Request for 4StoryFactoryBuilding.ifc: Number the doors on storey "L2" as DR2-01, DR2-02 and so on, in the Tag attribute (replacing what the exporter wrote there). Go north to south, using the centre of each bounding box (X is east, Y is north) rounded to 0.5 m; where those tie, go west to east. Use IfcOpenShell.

First a look at what the model holds.

```python
import ifcopenshell
import ifcopenshell.util.element
import ifcopenshell.util.placement

model = ifcopenshell.open("4StoryFactoryBuilding.ifc")
print(model.schema)
storey = next(s for s in model.by_type("IfcBuildingStorey") if s.Name == "L2")
doors = [e for e in ifcopenshell.util.element.get_decomposition(storey) if e.is_a("IfcDoor")]
for e in sorted(doors, key=lambda e: e.id()):
    origin = ifcopenshell.util.placement.get_local_placement(e.ObjectPlacement)[:3, 3]
    print(e.id(), e.Tag, e.Name, origin.round(2) + 0.0, sep=" | ")
```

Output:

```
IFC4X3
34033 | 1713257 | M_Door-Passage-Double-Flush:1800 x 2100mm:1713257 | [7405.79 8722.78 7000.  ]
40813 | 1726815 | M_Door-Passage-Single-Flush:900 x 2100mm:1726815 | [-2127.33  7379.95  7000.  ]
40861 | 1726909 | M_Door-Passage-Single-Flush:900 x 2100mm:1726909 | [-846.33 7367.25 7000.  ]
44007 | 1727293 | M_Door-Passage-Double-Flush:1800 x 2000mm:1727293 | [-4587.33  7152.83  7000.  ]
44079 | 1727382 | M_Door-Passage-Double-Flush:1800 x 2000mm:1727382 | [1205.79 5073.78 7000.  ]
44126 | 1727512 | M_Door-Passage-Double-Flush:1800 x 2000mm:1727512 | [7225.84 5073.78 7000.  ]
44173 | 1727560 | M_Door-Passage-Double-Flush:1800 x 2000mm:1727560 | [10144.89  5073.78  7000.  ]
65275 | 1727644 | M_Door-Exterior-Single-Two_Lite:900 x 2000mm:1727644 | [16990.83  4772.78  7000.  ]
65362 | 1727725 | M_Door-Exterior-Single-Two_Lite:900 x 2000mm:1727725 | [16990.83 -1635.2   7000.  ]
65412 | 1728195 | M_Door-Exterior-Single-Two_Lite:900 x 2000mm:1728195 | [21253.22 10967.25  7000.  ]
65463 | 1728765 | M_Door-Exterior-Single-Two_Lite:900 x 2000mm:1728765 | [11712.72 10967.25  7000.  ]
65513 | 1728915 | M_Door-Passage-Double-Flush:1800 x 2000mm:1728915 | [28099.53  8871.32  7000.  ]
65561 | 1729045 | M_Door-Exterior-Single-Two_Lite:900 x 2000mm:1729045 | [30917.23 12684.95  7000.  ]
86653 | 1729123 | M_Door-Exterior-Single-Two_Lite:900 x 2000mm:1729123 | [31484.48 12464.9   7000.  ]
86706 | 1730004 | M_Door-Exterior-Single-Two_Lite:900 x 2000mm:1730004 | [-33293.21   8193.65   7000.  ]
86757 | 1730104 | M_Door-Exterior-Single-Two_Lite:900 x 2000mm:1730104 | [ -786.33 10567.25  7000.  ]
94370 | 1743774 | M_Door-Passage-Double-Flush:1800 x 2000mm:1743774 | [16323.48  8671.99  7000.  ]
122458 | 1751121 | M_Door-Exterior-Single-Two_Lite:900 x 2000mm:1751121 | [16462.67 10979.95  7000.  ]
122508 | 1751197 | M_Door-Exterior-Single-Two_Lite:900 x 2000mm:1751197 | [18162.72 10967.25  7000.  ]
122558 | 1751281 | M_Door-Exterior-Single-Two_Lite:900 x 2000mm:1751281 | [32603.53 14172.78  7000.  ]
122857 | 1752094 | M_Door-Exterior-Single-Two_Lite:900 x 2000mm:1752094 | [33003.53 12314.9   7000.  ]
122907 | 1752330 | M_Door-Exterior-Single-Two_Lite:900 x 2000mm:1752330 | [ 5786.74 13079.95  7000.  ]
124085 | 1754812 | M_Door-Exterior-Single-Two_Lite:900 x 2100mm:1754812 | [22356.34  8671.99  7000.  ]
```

```python
import ifcopenshell
import ifcopenshell.geom
import ifcopenshell.util.element
import ifcopenshell.util.shape

model = ifcopenshell.open("4StoryFactoryBuilding.ifc")
settings = ifcopenshell.geom.settings()
settings.set("use-world-coords", True)


def centre(element):
    shape = ifcopenshell.geom.create_shape(settings, element)
    return ifcopenshell.util.shape.get_bbox_centroid(shape.geometry)


storey = next(s for s in model.by_type("IfcBuildingStorey") if s.Name == "L2")
doors = [e for e in ifcopenshell.util.element.get_decomposition(storey) if e.is_a("IfcDoor")]

# Insertion points can sit at a corner or the storey origin, so sort by the geometry (in metres).
centres = {e: centre(e) for e in doors}
doors.sort(key=lambda e: (-round(centres[e][1] / 0.5), centres[e][0]))

for i, e in enumerate(doors, start=1):
    number = f"DR2-{i:02d}"
    e.Tag = number
    print(e.id(), number)

model.write("4StoryFactoryBuilding-out.ifc")
```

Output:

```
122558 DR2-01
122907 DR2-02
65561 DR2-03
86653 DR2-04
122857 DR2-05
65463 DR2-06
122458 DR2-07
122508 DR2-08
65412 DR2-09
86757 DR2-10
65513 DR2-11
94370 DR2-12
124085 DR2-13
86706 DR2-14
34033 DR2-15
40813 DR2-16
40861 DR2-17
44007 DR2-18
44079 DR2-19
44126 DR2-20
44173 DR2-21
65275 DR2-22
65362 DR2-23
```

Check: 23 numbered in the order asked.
